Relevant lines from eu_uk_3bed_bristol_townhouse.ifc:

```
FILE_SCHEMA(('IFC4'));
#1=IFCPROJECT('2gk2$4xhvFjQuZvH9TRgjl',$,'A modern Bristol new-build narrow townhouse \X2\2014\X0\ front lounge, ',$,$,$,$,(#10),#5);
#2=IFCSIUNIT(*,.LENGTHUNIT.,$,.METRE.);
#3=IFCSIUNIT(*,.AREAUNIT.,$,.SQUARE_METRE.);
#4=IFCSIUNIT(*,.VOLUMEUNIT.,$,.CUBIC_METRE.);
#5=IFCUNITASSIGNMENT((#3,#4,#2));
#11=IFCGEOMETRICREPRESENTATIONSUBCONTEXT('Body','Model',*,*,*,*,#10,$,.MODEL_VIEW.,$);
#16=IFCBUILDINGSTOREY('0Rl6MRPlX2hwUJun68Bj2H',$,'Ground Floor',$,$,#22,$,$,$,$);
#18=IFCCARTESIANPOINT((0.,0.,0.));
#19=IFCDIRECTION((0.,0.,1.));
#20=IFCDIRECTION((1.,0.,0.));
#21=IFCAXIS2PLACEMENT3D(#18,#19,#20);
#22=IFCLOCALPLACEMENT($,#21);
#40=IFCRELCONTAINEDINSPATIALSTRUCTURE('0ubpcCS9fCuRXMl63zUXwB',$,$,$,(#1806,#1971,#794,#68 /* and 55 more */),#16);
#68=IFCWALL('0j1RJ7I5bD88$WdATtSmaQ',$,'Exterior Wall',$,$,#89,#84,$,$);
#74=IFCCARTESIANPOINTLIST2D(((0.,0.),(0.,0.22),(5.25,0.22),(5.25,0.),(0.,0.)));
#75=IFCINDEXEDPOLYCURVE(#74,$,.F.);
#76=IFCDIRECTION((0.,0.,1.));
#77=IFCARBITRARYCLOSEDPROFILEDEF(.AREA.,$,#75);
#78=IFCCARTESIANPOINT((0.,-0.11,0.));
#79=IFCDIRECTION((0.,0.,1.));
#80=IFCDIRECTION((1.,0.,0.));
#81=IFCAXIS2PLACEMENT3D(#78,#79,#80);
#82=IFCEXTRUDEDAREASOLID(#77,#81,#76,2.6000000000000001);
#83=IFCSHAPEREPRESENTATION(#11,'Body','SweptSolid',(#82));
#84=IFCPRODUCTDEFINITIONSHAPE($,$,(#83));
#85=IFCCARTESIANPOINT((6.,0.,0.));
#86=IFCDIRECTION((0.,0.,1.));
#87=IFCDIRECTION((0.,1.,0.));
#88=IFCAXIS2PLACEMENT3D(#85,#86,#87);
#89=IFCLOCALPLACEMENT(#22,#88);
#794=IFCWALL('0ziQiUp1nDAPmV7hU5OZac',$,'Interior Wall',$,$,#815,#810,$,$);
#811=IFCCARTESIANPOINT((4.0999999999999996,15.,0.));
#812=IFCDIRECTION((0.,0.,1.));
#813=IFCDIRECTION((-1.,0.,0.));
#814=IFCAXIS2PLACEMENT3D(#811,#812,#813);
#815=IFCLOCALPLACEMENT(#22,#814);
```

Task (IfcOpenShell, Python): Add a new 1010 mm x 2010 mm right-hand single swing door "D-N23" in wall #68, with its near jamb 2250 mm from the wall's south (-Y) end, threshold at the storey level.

```python
import numpy as np
import ifcopenshell
import ifcopenshell.api.feature
import ifcopenshell.api.geometry
import ifcopenshell.api.root
import ifcopenshell.api.spatial
import ifcopenshell.geom
import ifcopenshell.util.element
import ifcopenshell.util.placement
import ifcopenshell.util.representation
import ifcopenshell.util.shape
import ifcopenshell.util.unit

model = ifcopenshell.open("eu_uk_3bed_bristol_townhouse.ifc")
unit_scale = ifcopenshell.util.unit.calculate_unit_scale(model)
settings = ifcopenshell.geom.settings()


def volume(element):
    """Net volume in cubic metres, openings subtracted."""
    shape = ifcopenshell.geom.create_shape(settings, element)
    return ifcopenshell.util.shape.get_volume(shape.geometry)


wall = model.by_guid("0j1RJ7I5bD88$WdATtSmaQ")
storey = ifcopenshell.util.element.get_container(wall, ifc_class="IfcBuildingStorey")
context = ifcopenshell.util.representation.get_context(model, "Model", "Body", "MODEL_VIEW")
before = volume(wall)

width, height, from_end, sill = 1.01, 2.01, 2.25, 0.0  # metres

# The wall runs along its own X axis, and the end named is its -X end.
wall_shape = ifcopenshell.geom.create_shape(settings, wall)
x, y, z = ifcopenshell.util.shape.get_vertices(wall_shape.geometry).T
start = x.min() + from_end
face, thickness = float(y.min()), float(y.max() - y.min())
wall_matrix = ifcopenshell.util.placement.get_local_placement(wall.ObjectPlacement)
level = ifcopenshell.util.placement.get_local_placement(storey.ObjectPlacement)[2, 3]


def in_wall(x, y):
    """Placement at x, y metres in the wall's axes, at sill height."""
    matrix = wall_matrix.copy()
    matrix[:, 3] = wall_matrix @ np.array([x / unit_scale, y / unit_scale, 0.0, 1.0])
    matrix[2, 3] = level + sill / unit_scale
    return matrix


# Opening: a box that overshoots both wall faces by 50 mm.
opening = ifcopenshell.api.root.create_entity(model, ifc_class="IfcOpeningElement", predefined_type="OPENING")
box = ifcopenshell.api.geometry.add_wall_representation(
    model, context=context, length=width, height=height, thickness=thickness + 0.1
)
ifcopenshell.api.geometry.assign_representation(model, product=opening, representation=box)
ifcopenshell.api.geometry.edit_object_placement(model, product=opening, matrix=in_wall(start, face - 0.05), is_si=False)
ifcopenshell.api.feature.add_feature(model, feature=opening, element=wall)

door = ifcopenshell.api.root.create_entity(model, ifc_class="IfcDoor", name="D-N23", predefined_type="DOOR")
door.OverallWidth, door.OverallHeight = width / unit_scale, height / unit_scale
door.OperationType = "SINGLE_SWING_RIGHT"
body = ifcopenshell.api.geometry.add_door_representation(
    model,
    context=context,
    overall_width=door.OverallWidth,
    overall_height=door.OverallHeight,
    operation_type="SINGLE_SWING_RIGHT",
    lining_properties={"LiningDepth": thickness / unit_scale, "ThresholdDepth": thickness / unit_scale},
)
ifcopenshell.api.geometry.assign_representation(model, product=door, representation=body)
ifcopenshell.api.spatial.assign_container(model, products=[door], relating_structure=storey)
ifcopenshell.api.feature.add_filling(model, opening=opening, element=door)

# The lining spans the wall, so the door starts at the wall face.
ifcopenshell.api.geometry.edit_object_placement(model, product=door, matrix=in_wall(start, face), is_si=False)

after = volume(wall)

print(f"wall volume {before:.3f} -> {after:.3f} m3")

model.write("eu_uk_3bed_bristol_townhouse_edited.ifc")
```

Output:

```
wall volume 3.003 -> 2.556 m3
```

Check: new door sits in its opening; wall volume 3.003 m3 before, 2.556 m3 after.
